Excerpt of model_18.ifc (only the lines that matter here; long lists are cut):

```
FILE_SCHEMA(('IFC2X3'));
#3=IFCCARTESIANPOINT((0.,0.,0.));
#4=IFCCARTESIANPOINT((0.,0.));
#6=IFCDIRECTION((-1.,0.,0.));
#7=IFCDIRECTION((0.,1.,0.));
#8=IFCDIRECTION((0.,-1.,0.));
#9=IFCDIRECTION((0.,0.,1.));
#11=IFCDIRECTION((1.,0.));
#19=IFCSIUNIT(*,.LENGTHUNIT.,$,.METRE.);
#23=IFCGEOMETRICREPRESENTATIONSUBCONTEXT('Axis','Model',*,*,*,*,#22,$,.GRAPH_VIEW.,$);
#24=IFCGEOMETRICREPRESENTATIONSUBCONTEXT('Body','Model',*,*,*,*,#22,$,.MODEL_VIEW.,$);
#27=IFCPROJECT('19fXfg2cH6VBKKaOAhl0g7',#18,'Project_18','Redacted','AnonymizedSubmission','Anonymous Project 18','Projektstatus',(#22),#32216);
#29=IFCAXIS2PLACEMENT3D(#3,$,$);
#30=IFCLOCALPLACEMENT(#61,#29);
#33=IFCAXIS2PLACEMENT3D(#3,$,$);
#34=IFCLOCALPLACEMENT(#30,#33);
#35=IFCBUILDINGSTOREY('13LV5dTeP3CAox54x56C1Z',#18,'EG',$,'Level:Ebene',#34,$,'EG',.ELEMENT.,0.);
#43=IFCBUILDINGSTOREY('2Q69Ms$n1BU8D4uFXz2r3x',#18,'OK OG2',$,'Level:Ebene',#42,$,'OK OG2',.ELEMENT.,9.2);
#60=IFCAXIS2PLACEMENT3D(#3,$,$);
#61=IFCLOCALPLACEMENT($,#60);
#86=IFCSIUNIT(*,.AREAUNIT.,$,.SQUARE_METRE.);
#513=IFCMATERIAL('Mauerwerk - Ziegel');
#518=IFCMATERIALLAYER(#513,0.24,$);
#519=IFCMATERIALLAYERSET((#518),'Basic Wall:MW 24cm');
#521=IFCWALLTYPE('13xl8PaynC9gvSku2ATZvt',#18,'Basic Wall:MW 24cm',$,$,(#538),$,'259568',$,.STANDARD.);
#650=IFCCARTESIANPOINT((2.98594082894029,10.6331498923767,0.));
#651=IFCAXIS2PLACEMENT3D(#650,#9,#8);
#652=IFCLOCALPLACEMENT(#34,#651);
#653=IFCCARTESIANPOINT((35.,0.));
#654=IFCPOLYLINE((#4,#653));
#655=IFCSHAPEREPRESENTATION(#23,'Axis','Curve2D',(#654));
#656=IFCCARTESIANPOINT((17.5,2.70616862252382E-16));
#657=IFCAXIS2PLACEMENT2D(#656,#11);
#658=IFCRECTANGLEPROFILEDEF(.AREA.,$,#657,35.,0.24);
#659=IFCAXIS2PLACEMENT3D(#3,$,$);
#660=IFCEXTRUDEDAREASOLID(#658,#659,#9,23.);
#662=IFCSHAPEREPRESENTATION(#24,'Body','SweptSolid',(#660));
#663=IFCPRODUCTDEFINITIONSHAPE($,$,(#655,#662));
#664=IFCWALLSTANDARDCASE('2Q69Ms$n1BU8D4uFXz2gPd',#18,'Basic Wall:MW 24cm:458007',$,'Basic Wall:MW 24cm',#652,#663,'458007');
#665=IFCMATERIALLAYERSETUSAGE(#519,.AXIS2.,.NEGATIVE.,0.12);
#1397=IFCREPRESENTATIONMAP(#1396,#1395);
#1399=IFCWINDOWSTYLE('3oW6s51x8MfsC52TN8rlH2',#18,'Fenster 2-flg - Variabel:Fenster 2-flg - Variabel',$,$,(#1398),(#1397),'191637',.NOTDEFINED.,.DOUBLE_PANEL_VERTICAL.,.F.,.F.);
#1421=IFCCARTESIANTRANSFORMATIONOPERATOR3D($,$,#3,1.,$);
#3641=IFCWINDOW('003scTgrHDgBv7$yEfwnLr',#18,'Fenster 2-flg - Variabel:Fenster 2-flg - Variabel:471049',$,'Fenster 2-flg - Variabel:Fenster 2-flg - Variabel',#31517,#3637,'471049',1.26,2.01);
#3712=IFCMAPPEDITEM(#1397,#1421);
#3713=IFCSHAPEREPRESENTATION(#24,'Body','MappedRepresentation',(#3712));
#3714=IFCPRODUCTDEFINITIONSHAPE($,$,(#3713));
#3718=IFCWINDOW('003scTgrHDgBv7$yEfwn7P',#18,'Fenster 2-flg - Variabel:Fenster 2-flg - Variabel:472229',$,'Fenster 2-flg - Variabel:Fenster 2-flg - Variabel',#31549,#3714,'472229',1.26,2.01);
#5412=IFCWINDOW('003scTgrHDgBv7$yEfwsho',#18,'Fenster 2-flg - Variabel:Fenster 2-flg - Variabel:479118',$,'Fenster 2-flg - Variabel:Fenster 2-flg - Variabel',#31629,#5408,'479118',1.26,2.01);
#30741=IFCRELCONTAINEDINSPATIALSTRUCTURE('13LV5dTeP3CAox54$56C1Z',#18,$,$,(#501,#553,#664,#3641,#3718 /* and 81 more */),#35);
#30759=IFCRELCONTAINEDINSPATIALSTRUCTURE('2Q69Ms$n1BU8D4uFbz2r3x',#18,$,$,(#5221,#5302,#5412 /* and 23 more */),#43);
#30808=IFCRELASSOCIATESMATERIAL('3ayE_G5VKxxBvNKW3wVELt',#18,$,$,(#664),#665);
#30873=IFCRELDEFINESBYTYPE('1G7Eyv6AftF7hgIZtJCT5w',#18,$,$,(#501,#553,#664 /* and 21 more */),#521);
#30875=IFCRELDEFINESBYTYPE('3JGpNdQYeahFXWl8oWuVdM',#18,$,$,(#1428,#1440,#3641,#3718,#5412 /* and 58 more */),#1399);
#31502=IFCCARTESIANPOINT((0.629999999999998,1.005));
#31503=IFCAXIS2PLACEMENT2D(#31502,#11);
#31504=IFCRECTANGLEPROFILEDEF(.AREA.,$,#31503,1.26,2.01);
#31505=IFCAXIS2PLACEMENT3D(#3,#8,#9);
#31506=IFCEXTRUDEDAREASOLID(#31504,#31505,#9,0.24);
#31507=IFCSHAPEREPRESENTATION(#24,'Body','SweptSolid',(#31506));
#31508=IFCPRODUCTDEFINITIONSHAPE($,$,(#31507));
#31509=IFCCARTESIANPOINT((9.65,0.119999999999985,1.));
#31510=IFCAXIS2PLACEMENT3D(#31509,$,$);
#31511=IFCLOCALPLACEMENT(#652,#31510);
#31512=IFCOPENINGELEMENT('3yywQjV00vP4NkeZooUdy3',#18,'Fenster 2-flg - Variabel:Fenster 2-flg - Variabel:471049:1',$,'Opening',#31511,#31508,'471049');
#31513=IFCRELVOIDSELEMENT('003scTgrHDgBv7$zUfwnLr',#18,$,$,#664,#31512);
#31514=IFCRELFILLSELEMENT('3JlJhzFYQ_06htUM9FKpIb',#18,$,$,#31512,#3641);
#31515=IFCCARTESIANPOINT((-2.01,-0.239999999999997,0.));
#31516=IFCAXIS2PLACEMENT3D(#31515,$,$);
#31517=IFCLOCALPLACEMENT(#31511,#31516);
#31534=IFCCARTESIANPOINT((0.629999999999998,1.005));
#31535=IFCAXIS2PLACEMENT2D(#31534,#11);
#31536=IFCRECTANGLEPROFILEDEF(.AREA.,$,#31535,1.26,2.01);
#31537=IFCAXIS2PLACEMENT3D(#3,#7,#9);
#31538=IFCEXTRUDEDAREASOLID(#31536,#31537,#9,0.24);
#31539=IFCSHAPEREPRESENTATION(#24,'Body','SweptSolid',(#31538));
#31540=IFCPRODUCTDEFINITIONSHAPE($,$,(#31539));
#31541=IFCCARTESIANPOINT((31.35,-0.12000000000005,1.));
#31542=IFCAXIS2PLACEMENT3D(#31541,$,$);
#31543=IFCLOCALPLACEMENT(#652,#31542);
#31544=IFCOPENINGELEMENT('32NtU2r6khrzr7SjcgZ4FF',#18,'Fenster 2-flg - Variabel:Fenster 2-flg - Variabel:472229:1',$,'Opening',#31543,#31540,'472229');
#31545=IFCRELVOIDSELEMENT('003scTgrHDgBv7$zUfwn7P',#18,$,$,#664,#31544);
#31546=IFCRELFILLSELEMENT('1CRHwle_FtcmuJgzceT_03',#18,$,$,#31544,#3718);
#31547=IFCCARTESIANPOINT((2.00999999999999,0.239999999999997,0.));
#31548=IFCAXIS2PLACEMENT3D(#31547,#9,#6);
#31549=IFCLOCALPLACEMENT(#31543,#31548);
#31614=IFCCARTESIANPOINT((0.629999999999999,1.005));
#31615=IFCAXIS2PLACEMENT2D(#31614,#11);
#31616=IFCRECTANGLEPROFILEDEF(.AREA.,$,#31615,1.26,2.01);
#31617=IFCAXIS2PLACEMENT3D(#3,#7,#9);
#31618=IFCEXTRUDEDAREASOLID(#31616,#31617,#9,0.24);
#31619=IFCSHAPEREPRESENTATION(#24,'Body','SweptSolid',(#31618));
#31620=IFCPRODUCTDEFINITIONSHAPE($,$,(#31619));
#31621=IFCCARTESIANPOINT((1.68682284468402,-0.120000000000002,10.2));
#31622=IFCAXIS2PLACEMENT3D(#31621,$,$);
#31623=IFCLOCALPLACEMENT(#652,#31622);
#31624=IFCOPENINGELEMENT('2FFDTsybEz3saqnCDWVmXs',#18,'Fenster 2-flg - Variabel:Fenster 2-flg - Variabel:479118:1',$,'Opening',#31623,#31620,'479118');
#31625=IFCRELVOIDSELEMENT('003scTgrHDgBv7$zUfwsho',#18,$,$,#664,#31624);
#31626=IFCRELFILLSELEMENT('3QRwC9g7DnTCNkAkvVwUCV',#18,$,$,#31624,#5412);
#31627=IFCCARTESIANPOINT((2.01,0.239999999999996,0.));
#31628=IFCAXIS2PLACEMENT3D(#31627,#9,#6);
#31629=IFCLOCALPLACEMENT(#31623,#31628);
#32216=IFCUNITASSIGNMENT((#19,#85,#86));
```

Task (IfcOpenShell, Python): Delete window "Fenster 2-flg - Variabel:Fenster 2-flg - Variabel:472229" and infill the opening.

```python
import ifcopenshell
import ifcopenshell.api.feature
import ifcopenshell.api.root
import ifcopenshell.geom
import ifcopenshell.util.shape

model = ifcopenshell.open("model_18.ifc")
settings = ifcopenshell.geom.settings()


def volume(element):
    """Net volume in cubic metres, openings subtracted."""
    shape = ifcopenshell.geom.create_shape(settings, element)
    return ifcopenshell.util.shape.get_volume(shape.geometry)


window = model.by_guid("003scTgrHDgBv7$yEfwn7P")
opening = window.FillsVoids[0].RelatingOpeningElement
wall = opening.VoidsElements[0].RelatingBuildingElement
before = volume(wall)

ifcopenshell.api.root.remove_product(model, product=window)
ifcopenshell.api.feature.remove_feature(model, feature=opening)

after = volume(wall)

print(f"wall volume {before:.3f} -> {after:.3f} m3")

model.write("model_18_v2.ifc")
```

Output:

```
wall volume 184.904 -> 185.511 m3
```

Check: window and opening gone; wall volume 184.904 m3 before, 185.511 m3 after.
